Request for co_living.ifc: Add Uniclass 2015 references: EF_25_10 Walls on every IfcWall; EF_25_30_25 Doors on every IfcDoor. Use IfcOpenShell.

First a look at what the model holds.

```python
import ifcopenshell

model = ifcopenshell.open("co_living.ifc")
print(model.schema)
print("classifications:", [c.Name for c in model.by_type("IfcClassification")])
for ifc_class in ("IfcDoor", "IfcRoof", "IfcStair", "IfcWall", "IfcWindow"):
    print(ifc_class, len(model.by_type(ifc_class)))
```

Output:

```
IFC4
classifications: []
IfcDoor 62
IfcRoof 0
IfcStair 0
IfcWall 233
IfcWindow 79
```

```python
import ifcopenshell
import ifcopenshell.api.classification

model = ifcopenshell.open("co_living.ifc")

system = ifcopenshell.api.classification.add_classification(model, classification="Uniclass 2015")

codes = {
    "IfcWall": ("EF_25_10", "Walls"),
    "IfcDoor": ("EF_25_30_25", "Doors"),
}
for ifc_class, (code, name) in codes.items():
    products = model.by_type(ifc_class)
    ifcopenshell.api.classification.add_reference(
        model, products=products, classification=system, identification=code, name=name
    )
    print(code, len(products))

model.write("co_living_updated.ifc")
```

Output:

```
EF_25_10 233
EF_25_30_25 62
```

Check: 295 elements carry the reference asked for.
